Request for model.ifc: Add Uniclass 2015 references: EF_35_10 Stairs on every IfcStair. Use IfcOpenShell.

First a look at what the model holds.

```python
import ifcopenshell

model = ifcopenshell.open("model.ifc")
print(model.schema)
print("classifications:", [c.Name for c in model.by_type("IfcClassification")])
for ifc_class in ("IfcDoor", "IfcRoof", "IfcStair", "IfcWall", "IfcWindow"):
    print(ifc_class, len(model.by_type(ifc_class)))
```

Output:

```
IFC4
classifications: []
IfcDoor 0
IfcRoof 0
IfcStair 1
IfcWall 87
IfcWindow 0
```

```python
import ifcopenshell
import ifcopenshell.api.classification

model = ifcopenshell.open("model.ifc")

system = ifcopenshell.api.classification.add_classification(model, classification="Uniclass 2015")

codes = {
    "IfcStair": ("EF_35_10", "Stairs"),
}
for ifc_class, (code, name) in codes.items():
    products = model.by_type(ifc_class)
    ifcopenshell.api.classification.add_reference(
        model, products=products, classification=system, identification=code, name=name
    )
    print(code, len(products))

model.write("model_v2.ifc")
```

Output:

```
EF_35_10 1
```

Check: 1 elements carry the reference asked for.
